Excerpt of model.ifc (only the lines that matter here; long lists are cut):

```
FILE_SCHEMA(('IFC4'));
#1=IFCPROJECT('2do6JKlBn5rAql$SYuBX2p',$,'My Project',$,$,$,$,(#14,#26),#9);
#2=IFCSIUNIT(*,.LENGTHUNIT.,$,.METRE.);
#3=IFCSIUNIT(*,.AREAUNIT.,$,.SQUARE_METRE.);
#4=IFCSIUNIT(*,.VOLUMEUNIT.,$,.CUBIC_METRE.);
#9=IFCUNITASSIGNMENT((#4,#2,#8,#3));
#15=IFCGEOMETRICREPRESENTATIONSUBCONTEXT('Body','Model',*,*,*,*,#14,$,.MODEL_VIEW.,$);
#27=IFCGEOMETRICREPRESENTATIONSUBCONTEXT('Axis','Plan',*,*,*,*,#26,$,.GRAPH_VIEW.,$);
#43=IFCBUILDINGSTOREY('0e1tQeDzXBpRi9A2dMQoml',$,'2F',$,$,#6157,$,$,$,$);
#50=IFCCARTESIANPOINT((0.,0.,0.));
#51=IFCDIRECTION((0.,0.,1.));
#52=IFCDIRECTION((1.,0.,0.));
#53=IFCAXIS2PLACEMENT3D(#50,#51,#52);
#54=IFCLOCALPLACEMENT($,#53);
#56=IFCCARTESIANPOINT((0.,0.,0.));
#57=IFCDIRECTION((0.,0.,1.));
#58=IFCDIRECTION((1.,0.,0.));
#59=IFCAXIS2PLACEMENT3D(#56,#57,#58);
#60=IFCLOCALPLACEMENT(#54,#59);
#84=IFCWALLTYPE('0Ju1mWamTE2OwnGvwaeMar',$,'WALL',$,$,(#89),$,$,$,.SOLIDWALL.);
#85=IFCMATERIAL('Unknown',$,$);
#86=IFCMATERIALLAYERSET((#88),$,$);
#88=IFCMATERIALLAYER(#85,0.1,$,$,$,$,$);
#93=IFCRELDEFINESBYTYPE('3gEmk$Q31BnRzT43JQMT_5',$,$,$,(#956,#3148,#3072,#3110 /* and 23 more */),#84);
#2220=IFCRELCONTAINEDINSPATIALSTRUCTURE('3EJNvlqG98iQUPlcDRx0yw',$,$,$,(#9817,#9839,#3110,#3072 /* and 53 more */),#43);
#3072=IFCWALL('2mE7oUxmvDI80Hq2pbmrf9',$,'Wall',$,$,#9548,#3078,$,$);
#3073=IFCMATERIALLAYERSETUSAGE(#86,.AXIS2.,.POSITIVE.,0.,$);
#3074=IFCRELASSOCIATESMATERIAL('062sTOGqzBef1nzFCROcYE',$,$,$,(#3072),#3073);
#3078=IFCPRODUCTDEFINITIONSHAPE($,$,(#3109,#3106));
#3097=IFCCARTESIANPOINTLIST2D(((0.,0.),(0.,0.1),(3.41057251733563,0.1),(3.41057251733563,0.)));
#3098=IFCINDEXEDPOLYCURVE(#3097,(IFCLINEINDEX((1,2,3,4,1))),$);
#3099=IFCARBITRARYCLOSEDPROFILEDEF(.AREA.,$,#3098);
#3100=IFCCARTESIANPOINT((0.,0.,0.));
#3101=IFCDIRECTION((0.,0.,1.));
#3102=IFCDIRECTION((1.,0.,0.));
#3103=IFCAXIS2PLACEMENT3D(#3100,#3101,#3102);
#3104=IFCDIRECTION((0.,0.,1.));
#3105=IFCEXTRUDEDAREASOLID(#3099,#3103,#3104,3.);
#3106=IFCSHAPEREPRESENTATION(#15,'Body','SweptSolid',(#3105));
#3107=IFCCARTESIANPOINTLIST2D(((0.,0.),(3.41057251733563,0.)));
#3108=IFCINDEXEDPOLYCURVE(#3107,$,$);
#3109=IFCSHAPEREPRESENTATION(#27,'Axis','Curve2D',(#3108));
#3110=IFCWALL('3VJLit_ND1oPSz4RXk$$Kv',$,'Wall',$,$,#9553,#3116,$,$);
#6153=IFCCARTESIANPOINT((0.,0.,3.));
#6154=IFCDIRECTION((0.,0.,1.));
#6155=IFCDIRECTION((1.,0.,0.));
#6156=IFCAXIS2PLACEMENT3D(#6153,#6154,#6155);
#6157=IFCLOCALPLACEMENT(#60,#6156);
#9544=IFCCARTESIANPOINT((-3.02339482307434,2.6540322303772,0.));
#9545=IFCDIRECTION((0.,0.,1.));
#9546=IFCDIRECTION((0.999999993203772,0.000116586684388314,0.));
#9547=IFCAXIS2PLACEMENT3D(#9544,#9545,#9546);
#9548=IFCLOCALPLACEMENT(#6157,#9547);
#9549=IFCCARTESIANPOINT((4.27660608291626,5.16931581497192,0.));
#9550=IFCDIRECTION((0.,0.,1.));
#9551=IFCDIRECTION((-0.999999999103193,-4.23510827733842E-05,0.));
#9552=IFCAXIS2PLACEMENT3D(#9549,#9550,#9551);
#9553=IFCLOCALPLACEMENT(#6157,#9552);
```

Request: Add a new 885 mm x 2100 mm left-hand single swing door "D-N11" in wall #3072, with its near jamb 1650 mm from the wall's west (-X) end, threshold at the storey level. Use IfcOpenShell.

```python
import numpy as np
import ifcopenshell
import ifcopenshell.api.feature
import ifcopenshell.api.geometry
import ifcopenshell.api.root
import ifcopenshell.api.spatial
import ifcopenshell.geom
import ifcopenshell.util.element
import ifcopenshell.util.placement
import ifcopenshell.util.representation
import ifcopenshell.util.shape
import ifcopenshell.util.unit

model = ifcopenshell.open("model.ifc")
unit_scale = ifcopenshell.util.unit.calculate_unit_scale(model)
settings = ifcopenshell.geom.settings()


def volume(element):
    """Net volume in cubic metres, openings subtracted."""
    shape = ifcopenshell.geom.create_shape(settings, element)
    return ifcopenshell.util.shape.get_volume(shape.geometry)


wall = model.by_guid("2mE7oUxmvDI80Hq2pbmrf9")
storey = ifcopenshell.util.element.get_container(wall, ifc_class="IfcBuildingStorey")
context = ifcopenshell.util.representation.get_context(model, "Model", "Body", "MODEL_VIEW")
before = volume(wall)

width, height, from_end, sill = 0.885, 2.1, 1.65, 0.0  # metres

# The wall runs along its own X axis, and the end named is its -X end.
wall_shape = ifcopenshell.geom.create_shape(settings, wall)
x, y, z = ifcopenshell.util.shape.get_vertices(wall_shape.geometry).T
start = x.min() + from_end
face, thickness = float(y.min()), float(y.max() - y.min())
wall_matrix = ifcopenshell.util.placement.get_local_placement(wall.ObjectPlacement)
level = ifcopenshell.util.placement.get_local_placement(storey.ObjectPlacement)[2, 3]


def in_wall(x, y):
    """Placement at x, y metres in the wall's axes, at sill height."""
    matrix = wall_matrix.copy()
    matrix[:, 3] = wall_matrix @ np.array([x / unit_scale, y / unit_scale, 0.0, 1.0])
    matrix[2, 3] = level + sill / unit_scale
    return matrix


# Opening: a box that overshoots both wall faces by 50 mm.
opening = ifcopenshell.api.root.create_entity(model, ifc_class="IfcOpeningElement", predefined_type="OPENING")
box = ifcopenshell.api.geometry.add_wall_representation(
    model, context=context, length=width, height=height, thickness=thickness + 0.1
)
ifcopenshell.api.geometry.assign_representation(model, product=opening, representation=box)
ifcopenshell.api.geometry.edit_object_placement(model, product=opening, matrix=in_wall(start, face - 0.05), is_si=False)
ifcopenshell.api.feature.add_feature(model, feature=opening, element=wall)

door = ifcopenshell.api.root.create_entity(model, ifc_class="IfcDoor", name="D-N11", predefined_type="DOOR")
door.OverallWidth, door.OverallHeight = width / unit_scale, height / unit_scale
door.OperationType = "SINGLE_SWING_LEFT"
body = ifcopenshell.api.geometry.add_door_representation(
    model,
    context=context,
    overall_width=door.OverallWidth,
    overall_height=door.OverallHeight,
    operation_type="SINGLE_SWING_LEFT",
    lining_properties={"LiningDepth": thickness / unit_scale, "ThresholdDepth": thickness / unit_scale},
)
ifcopenshell.api.geometry.assign_representation(model, product=door, representation=body)
ifcopenshell.api.spatial.assign_container(model, products=[door], relating_structure=storey)
ifcopenshell.api.feature.add_filling(model, opening=opening, element=door)

# The lining spans the wall, so the door starts at the wall face.
ifcopenshell.api.geometry.edit_object_placement(model, product=door, matrix=in_wall(start, face), is_si=False)

after = volume(wall)

print(f"wall volume {before:.3f} -> {after:.3f} m3")

model.write("model-out.ifc")
```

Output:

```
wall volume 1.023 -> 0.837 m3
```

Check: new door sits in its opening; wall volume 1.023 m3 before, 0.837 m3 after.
